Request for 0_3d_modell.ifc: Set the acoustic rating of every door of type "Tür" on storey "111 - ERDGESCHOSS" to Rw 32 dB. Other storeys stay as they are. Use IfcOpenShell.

First a look at what the model holds.

```python
import ifcopenshell
import ifcopenshell.util.element

model = ifcopenshell.open("0_3d_modell.ifc")
print(model.schema)
storey = next(s for s in model.by_type("IfcBuildingStorey") if s.Name == "111 - ERDGESCHOSS")
doors = [e for e in ifcopenshell.util.element.get_decomposition(storey) if e.is_a("IfcDoor")]
seen = {}
for e in doors:
    element_type = ifcopenshell.util.element.get_type(e)
    key = (element_type.Name if element_type != e and element_type else None, ifcopenshell.util.element.get_pset(e, "Pset_DoorCommon", "AcousticRating"))
    seen[key] = seen.get(key, 0) + 1
for (name, value), count in sorted(seen.items(), key=str):
    print(count, "x", name, "|", value)
```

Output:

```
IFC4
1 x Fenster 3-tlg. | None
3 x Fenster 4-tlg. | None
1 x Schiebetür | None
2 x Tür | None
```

```python
import ifcopenshell
import ifcopenshell.api.pset
import ifcopenshell.util.element

model = ifcopenshell.open("0_3d_modell.ifc")

storey = next(s for s in model.by_type("IfcBuildingStorey") if s.Name == "111 - ERDGESCHOSS")
doors = [e for e in ifcopenshell.util.element.get_decomposition(storey) if e.is_a("IfcDoor")]

count = 0
for e in doors:
    element_type = ifcopenshell.util.element.get_type(e)
    if element_type in (None, e) or element_type.Name != "Tür":
        continue
    # add_pset returns the element's existing set when there is one.
    pset = ifcopenshell.api.pset.add_pset(model, product=e, name="Pset_DoorCommon")
    ifcopenshell.api.pset.edit_pset(model, pset=pset, properties={"AcousticRating": "Rw 32 dB"})
    count += 1

print(count, "doors updated")

model.write("0_3d_modell-out.ifc")
```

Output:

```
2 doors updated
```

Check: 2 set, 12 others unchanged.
